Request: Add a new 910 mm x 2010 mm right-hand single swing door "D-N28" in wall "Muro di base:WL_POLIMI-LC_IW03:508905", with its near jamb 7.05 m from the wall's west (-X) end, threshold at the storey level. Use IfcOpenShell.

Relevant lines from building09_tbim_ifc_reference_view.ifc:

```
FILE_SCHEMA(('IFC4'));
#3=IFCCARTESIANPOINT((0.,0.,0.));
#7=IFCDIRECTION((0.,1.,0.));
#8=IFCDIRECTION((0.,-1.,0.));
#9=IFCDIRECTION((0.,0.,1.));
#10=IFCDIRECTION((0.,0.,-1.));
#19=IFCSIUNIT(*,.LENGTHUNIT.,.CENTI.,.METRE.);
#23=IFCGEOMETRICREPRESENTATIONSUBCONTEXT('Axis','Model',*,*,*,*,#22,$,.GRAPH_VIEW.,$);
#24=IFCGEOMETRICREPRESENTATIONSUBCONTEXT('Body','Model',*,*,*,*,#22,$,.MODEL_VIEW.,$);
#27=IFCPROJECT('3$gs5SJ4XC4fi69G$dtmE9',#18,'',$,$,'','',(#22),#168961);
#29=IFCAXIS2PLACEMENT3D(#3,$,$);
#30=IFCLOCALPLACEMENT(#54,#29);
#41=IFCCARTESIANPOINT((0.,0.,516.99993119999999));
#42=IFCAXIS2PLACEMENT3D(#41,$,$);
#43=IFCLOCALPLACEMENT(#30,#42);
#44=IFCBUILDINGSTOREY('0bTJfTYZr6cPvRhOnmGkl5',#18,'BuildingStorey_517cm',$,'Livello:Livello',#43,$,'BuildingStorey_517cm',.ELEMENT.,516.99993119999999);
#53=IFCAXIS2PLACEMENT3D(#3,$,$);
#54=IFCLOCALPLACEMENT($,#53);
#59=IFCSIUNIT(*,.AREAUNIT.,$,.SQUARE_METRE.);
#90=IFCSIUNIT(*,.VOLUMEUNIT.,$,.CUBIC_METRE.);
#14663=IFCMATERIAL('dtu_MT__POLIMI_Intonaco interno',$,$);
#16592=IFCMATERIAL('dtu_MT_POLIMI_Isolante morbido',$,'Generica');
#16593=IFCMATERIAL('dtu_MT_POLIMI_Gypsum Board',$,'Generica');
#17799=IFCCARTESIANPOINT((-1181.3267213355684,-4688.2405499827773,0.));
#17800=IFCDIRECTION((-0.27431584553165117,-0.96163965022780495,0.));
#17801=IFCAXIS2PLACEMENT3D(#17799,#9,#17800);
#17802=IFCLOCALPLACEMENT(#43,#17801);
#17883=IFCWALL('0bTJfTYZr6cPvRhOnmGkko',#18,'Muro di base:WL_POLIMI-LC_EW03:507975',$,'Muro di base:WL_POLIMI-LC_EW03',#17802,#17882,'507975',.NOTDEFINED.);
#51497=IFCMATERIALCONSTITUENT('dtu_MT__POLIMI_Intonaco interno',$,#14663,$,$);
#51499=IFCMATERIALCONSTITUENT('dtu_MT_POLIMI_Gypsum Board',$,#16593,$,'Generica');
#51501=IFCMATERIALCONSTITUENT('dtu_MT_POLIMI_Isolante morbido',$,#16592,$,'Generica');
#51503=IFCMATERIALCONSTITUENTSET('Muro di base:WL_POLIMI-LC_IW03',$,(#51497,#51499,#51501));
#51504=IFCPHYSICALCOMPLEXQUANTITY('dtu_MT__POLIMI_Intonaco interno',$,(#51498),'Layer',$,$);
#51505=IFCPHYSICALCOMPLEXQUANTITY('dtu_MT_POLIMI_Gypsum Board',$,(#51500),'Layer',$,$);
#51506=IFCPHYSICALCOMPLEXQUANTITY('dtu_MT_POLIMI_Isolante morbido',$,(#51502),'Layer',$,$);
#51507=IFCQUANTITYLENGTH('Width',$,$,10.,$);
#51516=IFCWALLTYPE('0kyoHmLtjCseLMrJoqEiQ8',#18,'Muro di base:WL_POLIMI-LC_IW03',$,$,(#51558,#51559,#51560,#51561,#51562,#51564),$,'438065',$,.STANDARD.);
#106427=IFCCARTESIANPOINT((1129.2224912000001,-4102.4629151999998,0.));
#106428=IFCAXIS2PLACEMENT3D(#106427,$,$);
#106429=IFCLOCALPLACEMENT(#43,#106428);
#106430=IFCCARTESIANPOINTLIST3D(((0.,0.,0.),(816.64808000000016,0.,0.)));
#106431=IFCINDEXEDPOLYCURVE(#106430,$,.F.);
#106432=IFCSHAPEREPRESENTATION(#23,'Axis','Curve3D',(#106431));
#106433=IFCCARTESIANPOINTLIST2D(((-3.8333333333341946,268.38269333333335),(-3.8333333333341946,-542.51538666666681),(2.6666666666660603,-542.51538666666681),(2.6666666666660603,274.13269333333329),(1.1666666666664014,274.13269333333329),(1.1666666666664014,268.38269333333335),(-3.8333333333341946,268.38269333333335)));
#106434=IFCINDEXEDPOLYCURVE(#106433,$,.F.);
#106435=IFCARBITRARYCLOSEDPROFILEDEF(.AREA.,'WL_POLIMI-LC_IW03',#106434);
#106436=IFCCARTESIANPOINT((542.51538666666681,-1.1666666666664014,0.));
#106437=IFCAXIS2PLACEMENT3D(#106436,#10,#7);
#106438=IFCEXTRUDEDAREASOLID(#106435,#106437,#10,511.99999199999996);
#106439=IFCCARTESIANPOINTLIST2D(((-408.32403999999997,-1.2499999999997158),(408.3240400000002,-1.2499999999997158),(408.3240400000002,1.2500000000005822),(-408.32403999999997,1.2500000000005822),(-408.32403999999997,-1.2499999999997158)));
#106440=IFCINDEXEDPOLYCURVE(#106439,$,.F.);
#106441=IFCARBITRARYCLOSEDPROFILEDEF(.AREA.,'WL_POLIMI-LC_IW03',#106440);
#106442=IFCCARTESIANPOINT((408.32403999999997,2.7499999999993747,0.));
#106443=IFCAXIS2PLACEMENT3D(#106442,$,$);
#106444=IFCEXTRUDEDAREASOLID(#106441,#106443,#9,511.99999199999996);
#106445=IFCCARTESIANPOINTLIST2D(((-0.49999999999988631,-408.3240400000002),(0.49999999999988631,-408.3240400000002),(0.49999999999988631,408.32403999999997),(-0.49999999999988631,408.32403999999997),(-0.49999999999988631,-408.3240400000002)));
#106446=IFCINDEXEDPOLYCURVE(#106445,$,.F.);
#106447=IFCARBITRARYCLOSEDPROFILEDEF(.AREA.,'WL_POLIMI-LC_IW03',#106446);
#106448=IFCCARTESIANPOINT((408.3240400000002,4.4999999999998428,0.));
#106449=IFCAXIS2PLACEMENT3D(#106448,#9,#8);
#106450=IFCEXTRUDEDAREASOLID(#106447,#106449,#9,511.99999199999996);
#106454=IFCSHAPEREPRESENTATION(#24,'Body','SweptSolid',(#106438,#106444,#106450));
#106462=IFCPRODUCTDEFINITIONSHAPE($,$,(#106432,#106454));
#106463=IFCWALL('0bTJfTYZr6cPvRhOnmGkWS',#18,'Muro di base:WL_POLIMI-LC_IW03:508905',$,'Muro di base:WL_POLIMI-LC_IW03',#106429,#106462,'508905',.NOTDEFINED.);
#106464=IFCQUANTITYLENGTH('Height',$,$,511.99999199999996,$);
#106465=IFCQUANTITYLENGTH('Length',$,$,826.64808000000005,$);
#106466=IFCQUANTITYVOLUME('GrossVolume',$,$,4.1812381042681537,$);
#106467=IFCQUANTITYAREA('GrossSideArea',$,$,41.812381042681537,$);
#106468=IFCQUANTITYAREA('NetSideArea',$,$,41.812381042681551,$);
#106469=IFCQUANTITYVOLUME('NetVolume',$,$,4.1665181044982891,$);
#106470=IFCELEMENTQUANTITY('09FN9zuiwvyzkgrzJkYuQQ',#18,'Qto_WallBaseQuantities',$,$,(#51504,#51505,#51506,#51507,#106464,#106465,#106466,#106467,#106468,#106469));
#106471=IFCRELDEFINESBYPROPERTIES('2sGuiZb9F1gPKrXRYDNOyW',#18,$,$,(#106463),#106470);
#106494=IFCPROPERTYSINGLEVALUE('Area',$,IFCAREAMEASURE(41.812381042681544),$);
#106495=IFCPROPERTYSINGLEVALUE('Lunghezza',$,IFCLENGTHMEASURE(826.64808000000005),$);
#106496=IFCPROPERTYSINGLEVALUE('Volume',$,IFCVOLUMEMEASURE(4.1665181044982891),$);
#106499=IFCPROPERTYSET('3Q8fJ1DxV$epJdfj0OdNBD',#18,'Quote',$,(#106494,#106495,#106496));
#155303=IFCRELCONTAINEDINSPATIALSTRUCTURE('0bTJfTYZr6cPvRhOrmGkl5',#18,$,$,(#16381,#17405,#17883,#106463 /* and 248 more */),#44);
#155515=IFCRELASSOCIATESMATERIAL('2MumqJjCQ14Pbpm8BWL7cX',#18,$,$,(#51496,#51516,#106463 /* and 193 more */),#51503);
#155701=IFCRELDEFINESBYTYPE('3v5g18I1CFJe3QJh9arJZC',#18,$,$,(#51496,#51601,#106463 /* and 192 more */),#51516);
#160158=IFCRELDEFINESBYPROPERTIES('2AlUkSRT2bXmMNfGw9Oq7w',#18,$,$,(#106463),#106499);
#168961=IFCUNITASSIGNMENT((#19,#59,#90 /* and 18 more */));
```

```python
import numpy as np
import ifcopenshell
import ifcopenshell.api.feature
import ifcopenshell.api.geometry
import ifcopenshell.api.pset
import ifcopenshell.api.root
import ifcopenshell.api.spatial
import ifcopenshell.geom
import ifcopenshell.util.element
import ifcopenshell.util.placement
import ifcopenshell.util.representation
import ifcopenshell.util.shape
import ifcopenshell.util.unit

model = ifcopenshell.open("building09_tbim_ifc_reference_view.ifc")
unit_scale = ifcopenshell.util.unit.calculate_unit_scale(model)
area_scale = ifcopenshell.util.unit.calculate_unit_scale(model, "AREAUNIT")
volume_scale = ifcopenshell.util.unit.calculate_unit_scale(model, "VOLUMEUNIT")
settings = ifcopenshell.geom.settings()


def volume(element):
    """Net volume in cubic metres, openings subtracted."""
    shape = ifcopenshell.geom.create_shape(settings, element)
    return ifcopenshell.util.shape.get_volume(shape.geometry)


wall = model.by_guid("0bTJfTYZr6cPvRhOnmGkWS")
storey = ifcopenshell.util.element.get_container(wall, ifc_class="IfcBuildingStorey")
context = ifcopenshell.util.representation.get_context(model, "Model", "Body", "MODEL_VIEW")
before = volume(wall)

width, height, from_end, sill = 0.91, 2.01, 7.05, 0.0  # metres

# The wall runs along its own X axis, and the end named is its -X end.
wall_shape = ifcopenshell.geom.create_shape(settings, wall)
x, y, z = ifcopenshell.util.shape.get_vertices(wall_shape.geometry).T
start = x.min() + from_end
face, thickness = float(y.min()), float(y.max() - y.min())
wall_matrix = ifcopenshell.util.placement.get_local_placement(wall.ObjectPlacement)
level = ifcopenshell.util.placement.get_local_placement(storey.ObjectPlacement)[2, 3]


def in_wall(x, y):
    """Placement at x, y metres in the wall's axes, at sill height."""
    matrix = wall_matrix.copy()
    matrix[:, 3] = wall_matrix @ np.array([x / unit_scale, y / unit_scale, 0.0, 1.0])
    matrix[2, 3] = level + sill / unit_scale
    return matrix


# Opening: a box that overshoots both wall faces by 50 mm.
opening = ifcopenshell.api.root.create_entity(model, ifc_class="IfcOpeningElement", predefined_type="OPENING")
box = ifcopenshell.api.geometry.add_wall_representation(
    model, context=context, length=width, height=height, thickness=thickness + 0.1
)
ifcopenshell.api.geometry.assign_representation(model, product=opening, representation=box)
ifcopenshell.api.geometry.edit_object_placement(model, product=opening, matrix=in_wall(start, face - 0.05), is_si=False)
ifcopenshell.api.feature.add_feature(model, feature=opening, element=wall)

door = ifcopenshell.api.root.create_entity(model, ifc_class="IfcDoor", name="D-N28", predefined_type="DOOR")
door.OverallWidth, door.OverallHeight = width / unit_scale, height / unit_scale
door.OperationType = "SINGLE_SWING_RIGHT"
body = ifcopenshell.api.geometry.add_door_representation(
    model,
    context=context,
    overall_width=door.OverallWidth,
    overall_height=door.OverallHeight,
    operation_type="SINGLE_SWING_RIGHT",
    lining_properties={"LiningDepth": thickness / unit_scale, "ThresholdDepth": thickness / unit_scale},
)
ifcopenshell.api.geometry.assign_representation(model, product=door, representation=body)
ifcopenshell.api.spatial.assign_container(model, products=[door], relating_structure=storey)
ifcopenshell.api.feature.add_filling(model, opening=opening, element=door)

# The lining spans the wall, so the door starts at the wall face.
ifcopenshell.api.geometry.edit_object_placement(model, product=door, matrix=in_wall(start, face), is_si=False)

after = volume(wall)

# Update the wall's stored quantities.
qto = model.by_id(ifcopenshell.util.element.get_pset(wall, "Qto_WallBaseQuantities", should_inherit=False)["id"])
ifcopenshell.api.pset.edit_qto(model, qto=qto, properties={
    "NetSideArea": after / thickness / area_scale,
    "NetVolume": after / volume_scale,
})
pset = model.by_id(ifcopenshell.util.element.get_pset(wall, "Quote", should_inherit=False)["id"])
ifcopenshell.api.pset.edit_pset(model, pset=pset, properties={
    "Area": model.create_entity("IfcAreaMeasure", after / thickness / area_scale),
    "Volume": model.create_entity("IfcVolumeMeasure", after / volume_scale),
})

print(f"wall volume {before:.3f} -> {after:.3f} m3")

model.write("building09_tbim_ifc_reference_view-out.ifc")
```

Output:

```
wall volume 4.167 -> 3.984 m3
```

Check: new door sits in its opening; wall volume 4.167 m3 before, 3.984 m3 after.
